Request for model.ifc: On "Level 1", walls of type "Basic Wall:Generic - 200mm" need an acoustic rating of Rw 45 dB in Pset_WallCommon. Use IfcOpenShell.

First a look at what the model holds.

```python
import ifcopenshell
import ifcopenshell.util.element

model = ifcopenshell.open("model.ifc")
print(model.schema)
storey = next(s for s in model.by_type("IfcBuildingStorey") if s.Name == "Level 1")
walls = [e for e in ifcopenshell.util.element.get_decomposition(storey) if e.is_a("IfcWall")]
seen = {}
for e in walls:
    element_type = ifcopenshell.util.element.get_type(e)
    key = (element_type.Name if element_type != e and element_type else None, ifcopenshell.util.element.get_pset(e, "Pset_WallCommon", "AcousticRating"))
    seen[key] = seen.get(key, 0) + 1
for (name, value), count in sorted(seen.items(), key=str):
    print(count, "x", name, "|", value)
```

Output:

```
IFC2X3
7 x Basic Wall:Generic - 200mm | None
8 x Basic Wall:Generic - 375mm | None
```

```python
import ifcopenshell
import ifcopenshell.api.pset
import ifcopenshell.util.element

model = ifcopenshell.open("model.ifc")

storey = next(s for s in model.by_type("IfcBuildingStorey") if s.Name == "Level 1")
walls = [e for e in ifcopenshell.util.element.get_decomposition(storey) if e.is_a("IfcWall")]

count = 0
for e in walls:
    element_type = ifcopenshell.util.element.get_type(e)
    if element_type in (None, e) or element_type.Name != "Basic Wall:Generic - 200mm":
        continue
    # add_pset returns the element's existing set when there is one.
    pset = ifcopenshell.api.pset.add_pset(model, product=e, name="Pset_WallCommon")
    ifcopenshell.api.pset.edit_pset(model, pset=pset, properties={"AcousticRating": "Rw 45 dB"})
    count += 1

print(count, "walls updated")

model.write("model-out.ifc")
```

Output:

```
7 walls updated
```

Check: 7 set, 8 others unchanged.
